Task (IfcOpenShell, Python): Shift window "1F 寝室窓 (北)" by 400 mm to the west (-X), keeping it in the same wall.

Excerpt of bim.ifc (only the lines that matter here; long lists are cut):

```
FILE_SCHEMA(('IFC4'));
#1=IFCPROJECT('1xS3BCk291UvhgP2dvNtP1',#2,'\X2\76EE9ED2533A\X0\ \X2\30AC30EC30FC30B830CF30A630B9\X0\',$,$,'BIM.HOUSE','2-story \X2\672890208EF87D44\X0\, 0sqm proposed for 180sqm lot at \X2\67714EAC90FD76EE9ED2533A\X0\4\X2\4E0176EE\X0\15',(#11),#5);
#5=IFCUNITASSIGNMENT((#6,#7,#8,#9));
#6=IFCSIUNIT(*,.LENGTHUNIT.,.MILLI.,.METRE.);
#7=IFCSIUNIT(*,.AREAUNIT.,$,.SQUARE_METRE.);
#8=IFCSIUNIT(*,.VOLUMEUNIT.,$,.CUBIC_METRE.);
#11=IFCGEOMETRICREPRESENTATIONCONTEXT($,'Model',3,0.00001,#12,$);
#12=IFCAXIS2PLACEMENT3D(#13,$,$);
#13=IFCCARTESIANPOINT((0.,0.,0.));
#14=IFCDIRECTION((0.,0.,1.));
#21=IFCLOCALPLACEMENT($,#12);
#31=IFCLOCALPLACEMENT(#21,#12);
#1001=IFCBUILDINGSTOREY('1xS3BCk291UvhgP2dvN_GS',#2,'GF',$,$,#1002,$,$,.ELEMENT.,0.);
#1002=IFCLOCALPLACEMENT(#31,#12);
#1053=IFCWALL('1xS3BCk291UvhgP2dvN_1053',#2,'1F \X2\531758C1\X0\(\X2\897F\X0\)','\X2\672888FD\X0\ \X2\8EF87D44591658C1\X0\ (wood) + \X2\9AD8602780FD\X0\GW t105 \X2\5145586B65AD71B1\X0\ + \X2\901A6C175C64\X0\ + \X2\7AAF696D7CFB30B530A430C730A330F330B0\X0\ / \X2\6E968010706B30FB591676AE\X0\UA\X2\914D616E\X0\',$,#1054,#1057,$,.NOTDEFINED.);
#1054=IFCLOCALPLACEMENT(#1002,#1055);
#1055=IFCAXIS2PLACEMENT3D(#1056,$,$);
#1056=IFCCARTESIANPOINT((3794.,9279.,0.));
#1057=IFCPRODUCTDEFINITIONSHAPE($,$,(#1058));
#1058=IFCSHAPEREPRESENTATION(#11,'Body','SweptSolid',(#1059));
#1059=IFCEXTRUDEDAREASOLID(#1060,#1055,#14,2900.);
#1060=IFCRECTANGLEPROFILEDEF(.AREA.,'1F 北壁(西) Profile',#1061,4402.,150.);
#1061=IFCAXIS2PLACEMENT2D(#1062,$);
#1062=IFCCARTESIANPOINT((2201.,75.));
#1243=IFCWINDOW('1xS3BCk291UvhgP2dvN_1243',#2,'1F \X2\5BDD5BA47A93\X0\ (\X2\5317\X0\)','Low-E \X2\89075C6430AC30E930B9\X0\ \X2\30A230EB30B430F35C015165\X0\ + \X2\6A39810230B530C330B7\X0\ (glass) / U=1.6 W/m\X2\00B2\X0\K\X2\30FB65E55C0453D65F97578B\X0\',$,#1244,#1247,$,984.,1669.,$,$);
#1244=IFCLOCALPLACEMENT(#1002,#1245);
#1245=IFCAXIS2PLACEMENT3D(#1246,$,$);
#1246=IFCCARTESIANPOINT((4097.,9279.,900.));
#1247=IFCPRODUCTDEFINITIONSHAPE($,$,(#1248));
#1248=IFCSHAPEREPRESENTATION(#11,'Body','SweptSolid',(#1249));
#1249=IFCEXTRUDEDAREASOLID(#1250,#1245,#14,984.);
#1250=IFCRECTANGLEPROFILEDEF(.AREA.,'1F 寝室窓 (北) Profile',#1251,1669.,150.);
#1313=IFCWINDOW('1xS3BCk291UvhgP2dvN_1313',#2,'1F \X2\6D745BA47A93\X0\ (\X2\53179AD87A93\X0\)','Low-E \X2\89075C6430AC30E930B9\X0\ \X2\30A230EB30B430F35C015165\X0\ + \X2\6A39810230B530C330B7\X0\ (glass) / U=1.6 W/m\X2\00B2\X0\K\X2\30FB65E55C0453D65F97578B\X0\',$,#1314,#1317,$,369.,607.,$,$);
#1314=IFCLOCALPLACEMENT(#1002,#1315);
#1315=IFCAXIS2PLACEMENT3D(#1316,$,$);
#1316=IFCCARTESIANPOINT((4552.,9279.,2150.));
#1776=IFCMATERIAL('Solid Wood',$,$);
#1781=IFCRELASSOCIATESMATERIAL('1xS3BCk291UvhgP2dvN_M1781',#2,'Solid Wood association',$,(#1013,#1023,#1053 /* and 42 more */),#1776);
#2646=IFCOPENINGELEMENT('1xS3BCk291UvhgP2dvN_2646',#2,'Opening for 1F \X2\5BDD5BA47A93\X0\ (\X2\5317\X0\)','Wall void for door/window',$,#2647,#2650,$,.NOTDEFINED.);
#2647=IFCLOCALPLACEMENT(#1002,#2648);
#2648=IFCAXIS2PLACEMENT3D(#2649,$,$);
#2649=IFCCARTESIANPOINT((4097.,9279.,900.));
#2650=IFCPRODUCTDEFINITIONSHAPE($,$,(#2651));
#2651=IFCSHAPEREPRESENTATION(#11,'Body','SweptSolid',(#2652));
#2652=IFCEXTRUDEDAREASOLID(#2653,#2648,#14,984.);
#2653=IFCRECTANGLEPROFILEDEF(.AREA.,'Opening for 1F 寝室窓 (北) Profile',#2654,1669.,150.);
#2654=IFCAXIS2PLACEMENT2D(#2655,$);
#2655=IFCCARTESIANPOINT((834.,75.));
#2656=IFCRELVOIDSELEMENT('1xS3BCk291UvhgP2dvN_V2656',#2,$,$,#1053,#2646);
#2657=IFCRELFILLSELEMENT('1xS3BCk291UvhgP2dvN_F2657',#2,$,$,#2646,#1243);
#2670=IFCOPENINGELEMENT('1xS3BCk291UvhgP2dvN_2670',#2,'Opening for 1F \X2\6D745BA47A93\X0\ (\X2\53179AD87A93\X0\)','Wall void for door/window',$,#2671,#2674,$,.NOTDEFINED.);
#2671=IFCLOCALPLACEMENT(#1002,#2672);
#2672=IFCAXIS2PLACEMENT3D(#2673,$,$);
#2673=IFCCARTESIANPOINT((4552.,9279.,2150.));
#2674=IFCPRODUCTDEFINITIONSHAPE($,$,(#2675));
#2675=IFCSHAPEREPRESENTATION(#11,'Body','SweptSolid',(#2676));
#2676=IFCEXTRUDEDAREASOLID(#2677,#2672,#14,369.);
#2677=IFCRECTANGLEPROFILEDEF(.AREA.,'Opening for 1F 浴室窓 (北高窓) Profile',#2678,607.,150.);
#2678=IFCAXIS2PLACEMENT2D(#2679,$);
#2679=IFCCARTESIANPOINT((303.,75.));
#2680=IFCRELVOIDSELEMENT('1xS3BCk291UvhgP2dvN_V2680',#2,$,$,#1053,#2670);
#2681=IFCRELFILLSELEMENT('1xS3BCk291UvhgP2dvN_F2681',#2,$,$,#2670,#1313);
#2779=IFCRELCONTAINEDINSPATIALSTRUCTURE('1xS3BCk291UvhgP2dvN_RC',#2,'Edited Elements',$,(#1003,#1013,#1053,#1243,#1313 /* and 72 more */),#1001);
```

```python
import ifcopenshell
import ifcopenshell.api.geometry
import ifcopenshell.util.placement
import ifcopenshell.util.unit

model = ifcopenshell.open("bim.ifc")
unit_scale = ifcopenshell.util.unit.calculate_unit_scale(model)

window = model.by_guid("1xS3BCk291UvhgP2dvN_1243")
opening = window.FillsVoids[0].RelatingOpeningElement
wall = opening.VoidsElements[0].RelatingBuildingElement

wall_matrix = ifcopenshell.util.placement.get_local_placement(wall.ObjectPlacement)
shift = wall_matrix[:3, 0] * -0.4 / unit_scale
before = ifcopenshell.util.placement.get_local_placement(window.ObjectPlacement)[:3, 3].copy()

# The window is not placed relative to its opening, so move both.
for product in (opening, window):
    matrix = ifcopenshell.util.placement.get_local_placement(product.ObjectPlacement)
    matrix[:3, 3] += shift
    ifcopenshell.api.geometry.edit_object_placement(model, product=product, matrix=matrix, is_si=False)

after = ifcopenshell.util.placement.get_local_placement(window.ObjectPlacement)[:3, 3]
print("window moved by", (after - before).round(3) + 0.0)

model.write("bim_rev.ifc")
```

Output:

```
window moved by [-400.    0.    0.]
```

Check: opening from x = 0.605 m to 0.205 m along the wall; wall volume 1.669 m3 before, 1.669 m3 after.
